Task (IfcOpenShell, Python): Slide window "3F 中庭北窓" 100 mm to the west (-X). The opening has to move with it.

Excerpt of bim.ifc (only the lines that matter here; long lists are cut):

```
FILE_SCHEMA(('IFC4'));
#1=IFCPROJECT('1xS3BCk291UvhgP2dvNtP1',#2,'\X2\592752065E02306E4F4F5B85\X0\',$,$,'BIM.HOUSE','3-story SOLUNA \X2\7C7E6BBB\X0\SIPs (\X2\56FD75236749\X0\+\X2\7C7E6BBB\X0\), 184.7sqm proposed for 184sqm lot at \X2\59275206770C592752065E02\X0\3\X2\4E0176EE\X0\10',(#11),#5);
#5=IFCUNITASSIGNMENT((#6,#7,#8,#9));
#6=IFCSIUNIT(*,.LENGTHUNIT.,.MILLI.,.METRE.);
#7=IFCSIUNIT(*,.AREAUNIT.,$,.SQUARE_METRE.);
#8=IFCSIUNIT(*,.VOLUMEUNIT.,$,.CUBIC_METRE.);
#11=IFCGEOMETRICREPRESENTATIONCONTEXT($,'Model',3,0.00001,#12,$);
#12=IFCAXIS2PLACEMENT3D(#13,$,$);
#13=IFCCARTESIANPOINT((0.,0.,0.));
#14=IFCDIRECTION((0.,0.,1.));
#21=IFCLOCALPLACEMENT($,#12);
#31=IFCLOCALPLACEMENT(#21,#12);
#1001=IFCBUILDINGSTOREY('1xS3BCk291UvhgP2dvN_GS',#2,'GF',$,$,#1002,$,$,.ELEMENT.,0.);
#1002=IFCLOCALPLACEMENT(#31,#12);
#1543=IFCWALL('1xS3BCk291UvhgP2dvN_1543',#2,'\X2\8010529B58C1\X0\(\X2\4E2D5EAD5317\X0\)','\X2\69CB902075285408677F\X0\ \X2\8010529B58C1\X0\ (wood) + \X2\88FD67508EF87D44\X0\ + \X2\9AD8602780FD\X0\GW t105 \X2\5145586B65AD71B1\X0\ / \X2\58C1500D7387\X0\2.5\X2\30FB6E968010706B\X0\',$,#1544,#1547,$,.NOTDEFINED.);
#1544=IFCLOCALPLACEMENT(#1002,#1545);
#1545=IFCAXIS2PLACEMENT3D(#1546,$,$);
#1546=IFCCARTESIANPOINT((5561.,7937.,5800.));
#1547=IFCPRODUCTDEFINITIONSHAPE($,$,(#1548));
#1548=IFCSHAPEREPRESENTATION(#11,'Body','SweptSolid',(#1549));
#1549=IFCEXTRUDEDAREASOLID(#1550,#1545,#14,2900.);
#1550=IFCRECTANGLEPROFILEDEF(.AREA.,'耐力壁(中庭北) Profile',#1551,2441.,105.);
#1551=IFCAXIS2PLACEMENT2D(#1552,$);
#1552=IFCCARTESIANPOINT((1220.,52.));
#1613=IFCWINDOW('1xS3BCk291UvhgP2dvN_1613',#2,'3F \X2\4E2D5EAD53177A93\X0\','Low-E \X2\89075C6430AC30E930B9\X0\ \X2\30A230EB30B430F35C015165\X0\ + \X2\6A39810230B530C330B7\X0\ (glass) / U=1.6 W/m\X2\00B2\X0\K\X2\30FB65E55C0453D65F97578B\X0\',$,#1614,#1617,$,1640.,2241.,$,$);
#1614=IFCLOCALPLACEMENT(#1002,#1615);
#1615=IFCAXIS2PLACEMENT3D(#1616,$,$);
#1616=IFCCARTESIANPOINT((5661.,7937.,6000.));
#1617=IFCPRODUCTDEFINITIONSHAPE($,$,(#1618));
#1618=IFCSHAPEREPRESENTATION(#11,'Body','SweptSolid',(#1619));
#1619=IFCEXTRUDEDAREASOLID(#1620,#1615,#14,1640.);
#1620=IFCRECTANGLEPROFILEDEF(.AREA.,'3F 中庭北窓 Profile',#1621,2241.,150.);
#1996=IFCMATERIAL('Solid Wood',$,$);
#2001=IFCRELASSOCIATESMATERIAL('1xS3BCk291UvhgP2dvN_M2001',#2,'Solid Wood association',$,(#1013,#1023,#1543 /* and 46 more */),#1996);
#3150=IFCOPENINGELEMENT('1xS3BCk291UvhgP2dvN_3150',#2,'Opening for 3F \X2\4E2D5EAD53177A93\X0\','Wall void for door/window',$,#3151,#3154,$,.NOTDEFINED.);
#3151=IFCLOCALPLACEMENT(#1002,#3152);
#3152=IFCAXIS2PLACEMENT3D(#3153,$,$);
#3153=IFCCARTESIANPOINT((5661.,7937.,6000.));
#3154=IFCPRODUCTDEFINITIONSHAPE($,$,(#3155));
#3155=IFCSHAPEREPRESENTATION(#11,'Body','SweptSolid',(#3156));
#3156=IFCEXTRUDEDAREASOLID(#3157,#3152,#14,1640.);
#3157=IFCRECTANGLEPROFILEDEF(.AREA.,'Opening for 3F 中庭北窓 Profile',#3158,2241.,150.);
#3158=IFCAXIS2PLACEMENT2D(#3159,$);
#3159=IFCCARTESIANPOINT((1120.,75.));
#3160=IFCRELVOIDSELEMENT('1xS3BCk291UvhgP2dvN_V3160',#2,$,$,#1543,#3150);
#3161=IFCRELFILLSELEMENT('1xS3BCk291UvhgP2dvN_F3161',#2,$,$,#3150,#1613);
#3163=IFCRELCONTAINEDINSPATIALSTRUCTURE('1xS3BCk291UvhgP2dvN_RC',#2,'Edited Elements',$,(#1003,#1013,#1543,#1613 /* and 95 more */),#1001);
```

```python
import ifcopenshell
import ifcopenshell.api.geometry
import ifcopenshell.util.placement

model = ifcopenshell.open("bim.ifc")

window = model.by_id(1613)
opening = window.FillsVoids[0].RelatingOpeningElement
wall = opening.VoidsElements[0].RelatingBuildingElement

wall_matrix = ifcopenshell.util.placement.get_local_placement(wall.ObjectPlacement)
shift = wall_matrix[:3, 0] * -100.0
before = ifcopenshell.util.placement.get_local_placement(window.ObjectPlacement)[:3, 3].copy()

# The window is not placed relative to its opening, so move both.
for product in (opening, window):
    matrix = ifcopenshell.util.placement.get_local_placement(product.ObjectPlacement)
    matrix[:3, 3] += shift
    ifcopenshell.api.geometry.edit_object_placement(model, product=product, matrix=matrix, is_si=False)

after = ifcopenshell.util.placement.get_local_placement(window.ObjectPlacement)[:3, 3]
print("window moved by", (after - before).round(3) + 0.0)

model.write("bim_rev.ifc")
```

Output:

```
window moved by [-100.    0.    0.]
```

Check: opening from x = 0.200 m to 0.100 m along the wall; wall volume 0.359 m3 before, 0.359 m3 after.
